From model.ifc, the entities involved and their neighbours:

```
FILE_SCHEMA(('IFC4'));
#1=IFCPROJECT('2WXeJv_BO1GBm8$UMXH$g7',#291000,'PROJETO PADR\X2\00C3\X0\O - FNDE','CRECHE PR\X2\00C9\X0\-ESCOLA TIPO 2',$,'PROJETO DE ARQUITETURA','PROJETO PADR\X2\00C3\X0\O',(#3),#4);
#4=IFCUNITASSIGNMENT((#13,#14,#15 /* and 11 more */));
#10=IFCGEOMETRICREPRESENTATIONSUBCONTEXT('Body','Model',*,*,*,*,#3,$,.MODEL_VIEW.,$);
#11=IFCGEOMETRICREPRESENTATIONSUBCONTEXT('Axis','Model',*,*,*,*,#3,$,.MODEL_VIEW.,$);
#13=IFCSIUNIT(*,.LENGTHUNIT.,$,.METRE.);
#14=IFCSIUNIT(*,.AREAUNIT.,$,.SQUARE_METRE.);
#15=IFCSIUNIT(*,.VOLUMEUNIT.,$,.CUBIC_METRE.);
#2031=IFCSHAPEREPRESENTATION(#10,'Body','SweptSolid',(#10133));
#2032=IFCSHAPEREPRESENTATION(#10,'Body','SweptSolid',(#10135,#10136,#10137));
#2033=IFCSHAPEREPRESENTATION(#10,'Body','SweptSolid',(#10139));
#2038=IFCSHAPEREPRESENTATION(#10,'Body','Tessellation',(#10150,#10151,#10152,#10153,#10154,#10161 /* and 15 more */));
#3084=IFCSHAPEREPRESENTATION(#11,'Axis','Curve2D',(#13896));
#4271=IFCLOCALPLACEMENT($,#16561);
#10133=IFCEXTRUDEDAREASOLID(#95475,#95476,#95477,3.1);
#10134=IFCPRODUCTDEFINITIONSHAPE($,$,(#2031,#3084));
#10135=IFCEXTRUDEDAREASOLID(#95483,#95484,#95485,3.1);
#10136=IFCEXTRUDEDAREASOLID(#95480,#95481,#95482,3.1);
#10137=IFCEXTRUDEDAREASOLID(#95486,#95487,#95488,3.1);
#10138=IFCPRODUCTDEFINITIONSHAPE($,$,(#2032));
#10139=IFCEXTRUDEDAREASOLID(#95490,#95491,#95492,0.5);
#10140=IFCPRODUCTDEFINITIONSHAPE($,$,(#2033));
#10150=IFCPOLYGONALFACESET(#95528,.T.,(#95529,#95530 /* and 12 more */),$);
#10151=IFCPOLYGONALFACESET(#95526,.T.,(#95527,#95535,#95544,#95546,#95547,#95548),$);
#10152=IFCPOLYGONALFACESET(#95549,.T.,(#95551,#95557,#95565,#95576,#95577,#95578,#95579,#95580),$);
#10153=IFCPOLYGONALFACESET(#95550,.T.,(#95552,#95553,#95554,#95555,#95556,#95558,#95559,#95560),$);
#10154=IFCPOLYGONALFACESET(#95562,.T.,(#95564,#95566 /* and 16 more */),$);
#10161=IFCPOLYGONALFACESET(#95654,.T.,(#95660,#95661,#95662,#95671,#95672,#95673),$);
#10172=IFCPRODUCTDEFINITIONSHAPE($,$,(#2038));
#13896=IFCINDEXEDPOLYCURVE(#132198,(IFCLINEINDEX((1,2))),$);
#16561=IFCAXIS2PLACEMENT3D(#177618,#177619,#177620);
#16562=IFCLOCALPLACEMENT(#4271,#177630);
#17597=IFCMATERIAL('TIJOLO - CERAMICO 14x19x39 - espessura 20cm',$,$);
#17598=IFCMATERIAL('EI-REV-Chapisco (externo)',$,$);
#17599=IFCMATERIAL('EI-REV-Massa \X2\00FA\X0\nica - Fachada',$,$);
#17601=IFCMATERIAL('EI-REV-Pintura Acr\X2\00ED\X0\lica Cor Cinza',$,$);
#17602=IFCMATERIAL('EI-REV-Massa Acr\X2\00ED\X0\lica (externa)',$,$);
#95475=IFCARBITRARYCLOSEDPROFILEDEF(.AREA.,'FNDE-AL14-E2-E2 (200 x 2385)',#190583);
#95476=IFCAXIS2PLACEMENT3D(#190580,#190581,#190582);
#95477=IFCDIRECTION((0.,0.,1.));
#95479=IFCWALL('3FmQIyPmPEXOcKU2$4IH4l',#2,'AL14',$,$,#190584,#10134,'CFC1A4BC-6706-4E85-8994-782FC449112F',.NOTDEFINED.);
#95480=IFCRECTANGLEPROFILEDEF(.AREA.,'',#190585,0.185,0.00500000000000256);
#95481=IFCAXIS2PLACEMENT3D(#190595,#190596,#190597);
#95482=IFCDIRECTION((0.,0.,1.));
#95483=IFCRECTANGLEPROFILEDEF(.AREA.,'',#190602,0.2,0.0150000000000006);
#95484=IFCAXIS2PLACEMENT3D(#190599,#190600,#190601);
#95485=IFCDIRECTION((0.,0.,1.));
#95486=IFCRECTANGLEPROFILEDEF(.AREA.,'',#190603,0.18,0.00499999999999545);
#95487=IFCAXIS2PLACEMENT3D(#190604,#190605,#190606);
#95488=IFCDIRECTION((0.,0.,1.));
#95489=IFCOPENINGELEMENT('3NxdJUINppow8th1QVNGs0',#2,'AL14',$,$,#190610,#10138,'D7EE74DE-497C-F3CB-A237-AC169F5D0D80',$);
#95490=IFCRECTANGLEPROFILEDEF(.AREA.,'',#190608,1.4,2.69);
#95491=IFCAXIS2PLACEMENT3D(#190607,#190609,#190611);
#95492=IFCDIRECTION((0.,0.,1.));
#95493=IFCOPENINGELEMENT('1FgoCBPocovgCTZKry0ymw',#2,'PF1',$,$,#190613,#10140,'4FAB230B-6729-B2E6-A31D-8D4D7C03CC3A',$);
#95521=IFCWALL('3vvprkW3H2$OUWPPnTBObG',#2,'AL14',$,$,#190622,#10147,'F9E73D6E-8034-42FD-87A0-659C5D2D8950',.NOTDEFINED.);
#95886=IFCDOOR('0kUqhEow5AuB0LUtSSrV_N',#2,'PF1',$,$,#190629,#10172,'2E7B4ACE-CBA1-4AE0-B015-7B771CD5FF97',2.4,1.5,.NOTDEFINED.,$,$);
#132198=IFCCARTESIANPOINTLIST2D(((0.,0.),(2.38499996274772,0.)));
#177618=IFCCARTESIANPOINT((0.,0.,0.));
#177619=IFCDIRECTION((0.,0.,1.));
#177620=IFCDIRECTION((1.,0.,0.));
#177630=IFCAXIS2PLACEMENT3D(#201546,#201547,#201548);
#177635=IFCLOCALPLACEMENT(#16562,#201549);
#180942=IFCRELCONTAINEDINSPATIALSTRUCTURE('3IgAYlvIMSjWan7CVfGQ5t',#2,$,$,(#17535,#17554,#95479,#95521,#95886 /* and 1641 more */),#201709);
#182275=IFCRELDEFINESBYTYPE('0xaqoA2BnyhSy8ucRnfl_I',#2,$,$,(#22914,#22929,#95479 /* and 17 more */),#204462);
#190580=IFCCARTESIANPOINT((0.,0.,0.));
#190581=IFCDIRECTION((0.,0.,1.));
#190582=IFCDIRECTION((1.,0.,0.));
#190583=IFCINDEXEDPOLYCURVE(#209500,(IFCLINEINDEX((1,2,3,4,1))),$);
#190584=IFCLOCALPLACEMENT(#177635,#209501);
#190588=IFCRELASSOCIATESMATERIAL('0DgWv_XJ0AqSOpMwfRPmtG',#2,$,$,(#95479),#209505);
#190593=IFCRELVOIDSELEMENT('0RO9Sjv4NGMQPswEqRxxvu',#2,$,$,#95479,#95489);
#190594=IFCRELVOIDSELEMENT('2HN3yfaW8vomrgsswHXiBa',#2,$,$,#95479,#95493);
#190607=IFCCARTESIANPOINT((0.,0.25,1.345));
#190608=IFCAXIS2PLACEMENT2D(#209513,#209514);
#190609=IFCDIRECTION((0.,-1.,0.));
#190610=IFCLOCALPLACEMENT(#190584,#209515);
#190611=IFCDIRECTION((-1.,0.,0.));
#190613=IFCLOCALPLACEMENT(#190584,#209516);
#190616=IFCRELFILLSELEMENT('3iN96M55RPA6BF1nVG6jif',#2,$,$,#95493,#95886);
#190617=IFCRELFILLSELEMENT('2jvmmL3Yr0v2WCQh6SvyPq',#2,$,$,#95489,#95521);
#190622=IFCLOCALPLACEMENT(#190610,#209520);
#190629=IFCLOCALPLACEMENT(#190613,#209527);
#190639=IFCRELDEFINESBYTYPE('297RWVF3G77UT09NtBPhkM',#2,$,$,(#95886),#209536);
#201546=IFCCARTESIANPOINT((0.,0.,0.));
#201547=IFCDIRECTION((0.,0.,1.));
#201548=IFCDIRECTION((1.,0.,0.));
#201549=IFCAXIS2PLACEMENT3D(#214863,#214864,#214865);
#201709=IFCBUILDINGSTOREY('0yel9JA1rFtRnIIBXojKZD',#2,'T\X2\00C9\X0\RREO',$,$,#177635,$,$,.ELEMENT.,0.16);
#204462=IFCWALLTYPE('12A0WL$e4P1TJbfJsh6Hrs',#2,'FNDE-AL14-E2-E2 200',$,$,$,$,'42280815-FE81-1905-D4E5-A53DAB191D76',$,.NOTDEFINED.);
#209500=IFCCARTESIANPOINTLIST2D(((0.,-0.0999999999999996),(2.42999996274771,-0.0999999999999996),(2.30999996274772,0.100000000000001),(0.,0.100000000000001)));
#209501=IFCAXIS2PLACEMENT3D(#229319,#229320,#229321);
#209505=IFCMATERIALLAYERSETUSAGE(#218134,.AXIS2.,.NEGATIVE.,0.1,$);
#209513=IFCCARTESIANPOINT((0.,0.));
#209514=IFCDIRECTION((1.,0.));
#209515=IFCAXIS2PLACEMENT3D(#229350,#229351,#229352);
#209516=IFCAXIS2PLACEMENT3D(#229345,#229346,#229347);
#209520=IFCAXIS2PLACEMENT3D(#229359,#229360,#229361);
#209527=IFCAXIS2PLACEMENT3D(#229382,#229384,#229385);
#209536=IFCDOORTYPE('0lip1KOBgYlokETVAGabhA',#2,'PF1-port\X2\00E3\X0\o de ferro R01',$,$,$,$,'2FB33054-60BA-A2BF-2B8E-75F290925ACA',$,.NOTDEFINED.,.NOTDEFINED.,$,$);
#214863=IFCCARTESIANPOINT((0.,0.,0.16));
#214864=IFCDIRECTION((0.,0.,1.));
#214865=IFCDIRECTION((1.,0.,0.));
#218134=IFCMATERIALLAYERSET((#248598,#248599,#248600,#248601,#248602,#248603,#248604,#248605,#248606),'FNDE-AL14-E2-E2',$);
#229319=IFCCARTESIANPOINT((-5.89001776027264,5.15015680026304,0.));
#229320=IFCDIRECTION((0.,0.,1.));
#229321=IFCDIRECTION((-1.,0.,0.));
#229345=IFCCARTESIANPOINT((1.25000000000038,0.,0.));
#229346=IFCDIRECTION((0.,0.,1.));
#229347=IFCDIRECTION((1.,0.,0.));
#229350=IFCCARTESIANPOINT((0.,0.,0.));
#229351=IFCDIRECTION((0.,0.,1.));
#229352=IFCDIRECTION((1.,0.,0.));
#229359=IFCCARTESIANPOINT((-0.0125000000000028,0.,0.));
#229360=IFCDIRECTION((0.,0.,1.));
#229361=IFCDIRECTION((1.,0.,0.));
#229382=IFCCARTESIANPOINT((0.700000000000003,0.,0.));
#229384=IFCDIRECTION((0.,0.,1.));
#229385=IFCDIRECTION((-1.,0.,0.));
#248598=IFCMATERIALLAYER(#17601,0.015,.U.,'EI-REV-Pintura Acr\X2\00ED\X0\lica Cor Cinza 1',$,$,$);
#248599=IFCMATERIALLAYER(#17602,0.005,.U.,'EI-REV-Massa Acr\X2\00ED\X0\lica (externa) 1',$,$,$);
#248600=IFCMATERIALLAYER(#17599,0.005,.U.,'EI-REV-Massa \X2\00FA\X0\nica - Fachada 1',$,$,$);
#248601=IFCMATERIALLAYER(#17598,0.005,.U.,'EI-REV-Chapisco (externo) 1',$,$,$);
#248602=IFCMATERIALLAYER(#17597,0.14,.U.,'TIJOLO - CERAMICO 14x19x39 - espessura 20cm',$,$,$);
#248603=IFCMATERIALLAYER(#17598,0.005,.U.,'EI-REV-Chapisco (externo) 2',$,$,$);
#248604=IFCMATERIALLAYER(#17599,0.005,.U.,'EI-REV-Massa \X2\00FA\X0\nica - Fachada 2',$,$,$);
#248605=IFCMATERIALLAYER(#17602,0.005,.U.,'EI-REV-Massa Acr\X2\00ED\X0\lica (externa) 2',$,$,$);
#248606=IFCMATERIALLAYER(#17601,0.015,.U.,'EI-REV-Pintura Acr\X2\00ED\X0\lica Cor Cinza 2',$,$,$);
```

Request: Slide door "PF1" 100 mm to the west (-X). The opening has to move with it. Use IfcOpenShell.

```python
import ifcopenshell
import ifcopenshell.api.geometry
import ifcopenshell.util.placement

model = ifcopenshell.open("model.ifc")

door = model.by_id(95886)
opening = door.FillsVoids[0].RelatingOpeningElement
wall = opening.VoidsElements[0].RelatingBuildingElement

wall_matrix = ifcopenshell.util.placement.get_local_placement(wall.ObjectPlacement)
shift = wall_matrix[:3, 0] * 0.1
before = ifcopenshell.util.placement.get_local_placement(door.ObjectPlacement)[:3, 3].copy()

# The door is placed relative to its opening, so it follows when the opening moves.
matrix = ifcopenshell.util.placement.get_local_placement(opening.ObjectPlacement)
matrix[:3, 3] += shift
ifcopenshell.api.geometry.edit_object_placement(
    model, product=opening, matrix=matrix, is_si=False, should_transform_children=True
)

after = ifcopenshell.util.placement.get_local_placement(door.ObjectPlacement)[:3, 3]
print("door moved by", (after - before).round(3) + 0.0)

model.write("model_rev.ifc")
```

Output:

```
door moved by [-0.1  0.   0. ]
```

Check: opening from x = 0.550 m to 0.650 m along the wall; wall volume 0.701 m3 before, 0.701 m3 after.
